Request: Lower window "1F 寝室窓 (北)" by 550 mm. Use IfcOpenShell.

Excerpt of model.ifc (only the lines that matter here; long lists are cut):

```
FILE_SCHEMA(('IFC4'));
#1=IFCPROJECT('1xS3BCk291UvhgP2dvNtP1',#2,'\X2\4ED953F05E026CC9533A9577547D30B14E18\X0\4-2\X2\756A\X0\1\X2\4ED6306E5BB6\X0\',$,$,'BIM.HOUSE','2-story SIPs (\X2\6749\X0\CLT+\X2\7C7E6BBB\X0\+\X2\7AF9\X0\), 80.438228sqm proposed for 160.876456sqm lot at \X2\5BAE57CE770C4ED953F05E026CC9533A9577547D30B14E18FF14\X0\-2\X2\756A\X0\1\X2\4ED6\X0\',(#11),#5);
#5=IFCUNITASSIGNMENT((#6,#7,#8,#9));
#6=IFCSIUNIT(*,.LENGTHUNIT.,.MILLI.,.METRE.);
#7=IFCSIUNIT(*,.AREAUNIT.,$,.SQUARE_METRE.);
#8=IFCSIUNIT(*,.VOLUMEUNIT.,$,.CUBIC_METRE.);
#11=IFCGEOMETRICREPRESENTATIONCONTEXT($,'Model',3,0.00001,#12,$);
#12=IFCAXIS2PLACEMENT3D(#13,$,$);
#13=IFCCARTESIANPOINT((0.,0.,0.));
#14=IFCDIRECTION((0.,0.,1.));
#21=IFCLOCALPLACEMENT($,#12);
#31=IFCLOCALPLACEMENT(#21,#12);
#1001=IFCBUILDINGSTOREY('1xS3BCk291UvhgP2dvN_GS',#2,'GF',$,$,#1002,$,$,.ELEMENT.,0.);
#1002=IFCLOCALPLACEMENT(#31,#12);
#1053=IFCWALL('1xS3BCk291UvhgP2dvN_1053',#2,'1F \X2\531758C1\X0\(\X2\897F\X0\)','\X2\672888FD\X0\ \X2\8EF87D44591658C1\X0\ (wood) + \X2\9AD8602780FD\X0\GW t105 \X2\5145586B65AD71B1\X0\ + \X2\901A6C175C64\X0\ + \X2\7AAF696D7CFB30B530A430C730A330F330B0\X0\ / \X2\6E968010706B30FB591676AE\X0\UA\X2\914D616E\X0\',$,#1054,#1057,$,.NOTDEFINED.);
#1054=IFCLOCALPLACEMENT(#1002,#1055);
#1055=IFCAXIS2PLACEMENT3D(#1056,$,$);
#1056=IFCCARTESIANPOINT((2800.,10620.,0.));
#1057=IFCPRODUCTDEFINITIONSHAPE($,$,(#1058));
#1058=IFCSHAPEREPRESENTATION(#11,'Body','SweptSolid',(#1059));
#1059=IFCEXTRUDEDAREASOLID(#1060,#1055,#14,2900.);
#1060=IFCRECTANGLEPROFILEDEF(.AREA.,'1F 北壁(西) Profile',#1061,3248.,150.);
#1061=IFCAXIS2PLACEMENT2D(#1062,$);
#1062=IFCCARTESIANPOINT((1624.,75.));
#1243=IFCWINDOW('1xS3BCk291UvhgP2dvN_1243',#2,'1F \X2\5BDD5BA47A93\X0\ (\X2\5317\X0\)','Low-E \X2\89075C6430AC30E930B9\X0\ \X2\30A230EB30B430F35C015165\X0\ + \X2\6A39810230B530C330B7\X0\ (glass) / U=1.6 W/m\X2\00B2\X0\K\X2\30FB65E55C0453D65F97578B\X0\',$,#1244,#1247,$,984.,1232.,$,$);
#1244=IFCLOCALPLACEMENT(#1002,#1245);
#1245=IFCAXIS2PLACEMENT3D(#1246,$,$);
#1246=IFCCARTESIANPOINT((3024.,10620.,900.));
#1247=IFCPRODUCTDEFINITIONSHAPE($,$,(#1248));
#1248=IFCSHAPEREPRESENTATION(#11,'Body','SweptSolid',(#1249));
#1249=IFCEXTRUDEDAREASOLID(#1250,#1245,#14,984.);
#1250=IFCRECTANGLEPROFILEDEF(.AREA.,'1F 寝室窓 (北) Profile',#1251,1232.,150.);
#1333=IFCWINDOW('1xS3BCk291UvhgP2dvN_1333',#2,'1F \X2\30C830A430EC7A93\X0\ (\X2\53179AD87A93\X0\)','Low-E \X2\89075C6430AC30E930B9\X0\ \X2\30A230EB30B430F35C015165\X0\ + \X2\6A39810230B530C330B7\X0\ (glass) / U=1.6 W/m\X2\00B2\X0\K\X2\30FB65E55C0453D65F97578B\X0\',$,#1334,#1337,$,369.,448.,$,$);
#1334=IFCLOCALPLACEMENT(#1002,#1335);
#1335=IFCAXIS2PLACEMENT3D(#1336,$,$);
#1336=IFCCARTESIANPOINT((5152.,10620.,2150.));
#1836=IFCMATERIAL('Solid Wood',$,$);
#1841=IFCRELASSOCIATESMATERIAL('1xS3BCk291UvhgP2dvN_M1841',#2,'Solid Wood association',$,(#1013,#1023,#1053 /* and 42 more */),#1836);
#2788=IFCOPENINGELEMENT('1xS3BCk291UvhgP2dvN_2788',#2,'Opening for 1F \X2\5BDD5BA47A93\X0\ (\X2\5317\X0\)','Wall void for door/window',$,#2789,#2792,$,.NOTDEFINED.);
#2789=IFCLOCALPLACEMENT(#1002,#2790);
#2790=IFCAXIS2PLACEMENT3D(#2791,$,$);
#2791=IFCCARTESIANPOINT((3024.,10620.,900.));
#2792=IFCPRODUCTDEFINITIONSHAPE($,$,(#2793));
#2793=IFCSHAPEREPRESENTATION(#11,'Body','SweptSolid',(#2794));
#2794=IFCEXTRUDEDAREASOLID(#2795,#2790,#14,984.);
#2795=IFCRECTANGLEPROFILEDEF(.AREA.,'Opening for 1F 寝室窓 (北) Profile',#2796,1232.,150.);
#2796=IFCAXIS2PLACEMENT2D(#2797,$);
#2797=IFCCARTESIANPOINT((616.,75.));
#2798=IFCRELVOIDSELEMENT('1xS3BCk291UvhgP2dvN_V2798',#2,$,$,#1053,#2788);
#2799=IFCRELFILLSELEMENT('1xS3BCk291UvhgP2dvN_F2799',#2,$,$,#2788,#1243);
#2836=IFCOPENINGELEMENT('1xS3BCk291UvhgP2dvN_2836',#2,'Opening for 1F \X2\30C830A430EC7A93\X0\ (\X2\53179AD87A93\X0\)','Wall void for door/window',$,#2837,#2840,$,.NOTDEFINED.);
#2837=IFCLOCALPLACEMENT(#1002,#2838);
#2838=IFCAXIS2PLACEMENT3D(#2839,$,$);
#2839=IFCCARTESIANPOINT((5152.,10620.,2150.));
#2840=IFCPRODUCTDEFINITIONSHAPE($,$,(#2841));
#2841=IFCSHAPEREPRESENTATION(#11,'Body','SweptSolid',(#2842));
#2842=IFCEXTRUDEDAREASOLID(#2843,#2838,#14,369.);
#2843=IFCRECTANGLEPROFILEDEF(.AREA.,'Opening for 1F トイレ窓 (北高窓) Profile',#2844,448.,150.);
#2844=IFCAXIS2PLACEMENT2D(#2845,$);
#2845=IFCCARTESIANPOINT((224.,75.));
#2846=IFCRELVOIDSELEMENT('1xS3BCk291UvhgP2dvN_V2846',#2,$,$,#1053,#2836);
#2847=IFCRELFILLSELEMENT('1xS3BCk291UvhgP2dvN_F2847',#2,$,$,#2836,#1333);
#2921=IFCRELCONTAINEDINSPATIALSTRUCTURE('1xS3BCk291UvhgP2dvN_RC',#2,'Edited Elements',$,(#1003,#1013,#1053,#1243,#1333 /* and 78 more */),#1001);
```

```python
import numpy as np
import ifcopenshell
import ifcopenshell.api.geometry
import ifcopenshell.util.placement
import ifcopenshell.util.unit

model = ifcopenshell.open("model.ifc")
unit_scale = ifcopenshell.util.unit.calculate_unit_scale(model)

window = model.by_id(1243)
opening = window.FillsVoids[0].RelatingOpeningElement
dz = -0.55 / unit_scale

shift = np.array([0.0, 0.0, dz])
# The window is not placed relative to its opening, so move both.
for product in (opening, window):
    matrix = ifcopenshell.util.placement.get_local_placement(product.ObjectPlacement)
    matrix[:3, 3] += shift
    ifcopenshell.api.geometry.edit_object_placement(model, product=product, matrix=matrix, is_si=False)

print(f"moved by {dz * unit_scale:+.3f} m")

model.write("model_updated.ifc")
```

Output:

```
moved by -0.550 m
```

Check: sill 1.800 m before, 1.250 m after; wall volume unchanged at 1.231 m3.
